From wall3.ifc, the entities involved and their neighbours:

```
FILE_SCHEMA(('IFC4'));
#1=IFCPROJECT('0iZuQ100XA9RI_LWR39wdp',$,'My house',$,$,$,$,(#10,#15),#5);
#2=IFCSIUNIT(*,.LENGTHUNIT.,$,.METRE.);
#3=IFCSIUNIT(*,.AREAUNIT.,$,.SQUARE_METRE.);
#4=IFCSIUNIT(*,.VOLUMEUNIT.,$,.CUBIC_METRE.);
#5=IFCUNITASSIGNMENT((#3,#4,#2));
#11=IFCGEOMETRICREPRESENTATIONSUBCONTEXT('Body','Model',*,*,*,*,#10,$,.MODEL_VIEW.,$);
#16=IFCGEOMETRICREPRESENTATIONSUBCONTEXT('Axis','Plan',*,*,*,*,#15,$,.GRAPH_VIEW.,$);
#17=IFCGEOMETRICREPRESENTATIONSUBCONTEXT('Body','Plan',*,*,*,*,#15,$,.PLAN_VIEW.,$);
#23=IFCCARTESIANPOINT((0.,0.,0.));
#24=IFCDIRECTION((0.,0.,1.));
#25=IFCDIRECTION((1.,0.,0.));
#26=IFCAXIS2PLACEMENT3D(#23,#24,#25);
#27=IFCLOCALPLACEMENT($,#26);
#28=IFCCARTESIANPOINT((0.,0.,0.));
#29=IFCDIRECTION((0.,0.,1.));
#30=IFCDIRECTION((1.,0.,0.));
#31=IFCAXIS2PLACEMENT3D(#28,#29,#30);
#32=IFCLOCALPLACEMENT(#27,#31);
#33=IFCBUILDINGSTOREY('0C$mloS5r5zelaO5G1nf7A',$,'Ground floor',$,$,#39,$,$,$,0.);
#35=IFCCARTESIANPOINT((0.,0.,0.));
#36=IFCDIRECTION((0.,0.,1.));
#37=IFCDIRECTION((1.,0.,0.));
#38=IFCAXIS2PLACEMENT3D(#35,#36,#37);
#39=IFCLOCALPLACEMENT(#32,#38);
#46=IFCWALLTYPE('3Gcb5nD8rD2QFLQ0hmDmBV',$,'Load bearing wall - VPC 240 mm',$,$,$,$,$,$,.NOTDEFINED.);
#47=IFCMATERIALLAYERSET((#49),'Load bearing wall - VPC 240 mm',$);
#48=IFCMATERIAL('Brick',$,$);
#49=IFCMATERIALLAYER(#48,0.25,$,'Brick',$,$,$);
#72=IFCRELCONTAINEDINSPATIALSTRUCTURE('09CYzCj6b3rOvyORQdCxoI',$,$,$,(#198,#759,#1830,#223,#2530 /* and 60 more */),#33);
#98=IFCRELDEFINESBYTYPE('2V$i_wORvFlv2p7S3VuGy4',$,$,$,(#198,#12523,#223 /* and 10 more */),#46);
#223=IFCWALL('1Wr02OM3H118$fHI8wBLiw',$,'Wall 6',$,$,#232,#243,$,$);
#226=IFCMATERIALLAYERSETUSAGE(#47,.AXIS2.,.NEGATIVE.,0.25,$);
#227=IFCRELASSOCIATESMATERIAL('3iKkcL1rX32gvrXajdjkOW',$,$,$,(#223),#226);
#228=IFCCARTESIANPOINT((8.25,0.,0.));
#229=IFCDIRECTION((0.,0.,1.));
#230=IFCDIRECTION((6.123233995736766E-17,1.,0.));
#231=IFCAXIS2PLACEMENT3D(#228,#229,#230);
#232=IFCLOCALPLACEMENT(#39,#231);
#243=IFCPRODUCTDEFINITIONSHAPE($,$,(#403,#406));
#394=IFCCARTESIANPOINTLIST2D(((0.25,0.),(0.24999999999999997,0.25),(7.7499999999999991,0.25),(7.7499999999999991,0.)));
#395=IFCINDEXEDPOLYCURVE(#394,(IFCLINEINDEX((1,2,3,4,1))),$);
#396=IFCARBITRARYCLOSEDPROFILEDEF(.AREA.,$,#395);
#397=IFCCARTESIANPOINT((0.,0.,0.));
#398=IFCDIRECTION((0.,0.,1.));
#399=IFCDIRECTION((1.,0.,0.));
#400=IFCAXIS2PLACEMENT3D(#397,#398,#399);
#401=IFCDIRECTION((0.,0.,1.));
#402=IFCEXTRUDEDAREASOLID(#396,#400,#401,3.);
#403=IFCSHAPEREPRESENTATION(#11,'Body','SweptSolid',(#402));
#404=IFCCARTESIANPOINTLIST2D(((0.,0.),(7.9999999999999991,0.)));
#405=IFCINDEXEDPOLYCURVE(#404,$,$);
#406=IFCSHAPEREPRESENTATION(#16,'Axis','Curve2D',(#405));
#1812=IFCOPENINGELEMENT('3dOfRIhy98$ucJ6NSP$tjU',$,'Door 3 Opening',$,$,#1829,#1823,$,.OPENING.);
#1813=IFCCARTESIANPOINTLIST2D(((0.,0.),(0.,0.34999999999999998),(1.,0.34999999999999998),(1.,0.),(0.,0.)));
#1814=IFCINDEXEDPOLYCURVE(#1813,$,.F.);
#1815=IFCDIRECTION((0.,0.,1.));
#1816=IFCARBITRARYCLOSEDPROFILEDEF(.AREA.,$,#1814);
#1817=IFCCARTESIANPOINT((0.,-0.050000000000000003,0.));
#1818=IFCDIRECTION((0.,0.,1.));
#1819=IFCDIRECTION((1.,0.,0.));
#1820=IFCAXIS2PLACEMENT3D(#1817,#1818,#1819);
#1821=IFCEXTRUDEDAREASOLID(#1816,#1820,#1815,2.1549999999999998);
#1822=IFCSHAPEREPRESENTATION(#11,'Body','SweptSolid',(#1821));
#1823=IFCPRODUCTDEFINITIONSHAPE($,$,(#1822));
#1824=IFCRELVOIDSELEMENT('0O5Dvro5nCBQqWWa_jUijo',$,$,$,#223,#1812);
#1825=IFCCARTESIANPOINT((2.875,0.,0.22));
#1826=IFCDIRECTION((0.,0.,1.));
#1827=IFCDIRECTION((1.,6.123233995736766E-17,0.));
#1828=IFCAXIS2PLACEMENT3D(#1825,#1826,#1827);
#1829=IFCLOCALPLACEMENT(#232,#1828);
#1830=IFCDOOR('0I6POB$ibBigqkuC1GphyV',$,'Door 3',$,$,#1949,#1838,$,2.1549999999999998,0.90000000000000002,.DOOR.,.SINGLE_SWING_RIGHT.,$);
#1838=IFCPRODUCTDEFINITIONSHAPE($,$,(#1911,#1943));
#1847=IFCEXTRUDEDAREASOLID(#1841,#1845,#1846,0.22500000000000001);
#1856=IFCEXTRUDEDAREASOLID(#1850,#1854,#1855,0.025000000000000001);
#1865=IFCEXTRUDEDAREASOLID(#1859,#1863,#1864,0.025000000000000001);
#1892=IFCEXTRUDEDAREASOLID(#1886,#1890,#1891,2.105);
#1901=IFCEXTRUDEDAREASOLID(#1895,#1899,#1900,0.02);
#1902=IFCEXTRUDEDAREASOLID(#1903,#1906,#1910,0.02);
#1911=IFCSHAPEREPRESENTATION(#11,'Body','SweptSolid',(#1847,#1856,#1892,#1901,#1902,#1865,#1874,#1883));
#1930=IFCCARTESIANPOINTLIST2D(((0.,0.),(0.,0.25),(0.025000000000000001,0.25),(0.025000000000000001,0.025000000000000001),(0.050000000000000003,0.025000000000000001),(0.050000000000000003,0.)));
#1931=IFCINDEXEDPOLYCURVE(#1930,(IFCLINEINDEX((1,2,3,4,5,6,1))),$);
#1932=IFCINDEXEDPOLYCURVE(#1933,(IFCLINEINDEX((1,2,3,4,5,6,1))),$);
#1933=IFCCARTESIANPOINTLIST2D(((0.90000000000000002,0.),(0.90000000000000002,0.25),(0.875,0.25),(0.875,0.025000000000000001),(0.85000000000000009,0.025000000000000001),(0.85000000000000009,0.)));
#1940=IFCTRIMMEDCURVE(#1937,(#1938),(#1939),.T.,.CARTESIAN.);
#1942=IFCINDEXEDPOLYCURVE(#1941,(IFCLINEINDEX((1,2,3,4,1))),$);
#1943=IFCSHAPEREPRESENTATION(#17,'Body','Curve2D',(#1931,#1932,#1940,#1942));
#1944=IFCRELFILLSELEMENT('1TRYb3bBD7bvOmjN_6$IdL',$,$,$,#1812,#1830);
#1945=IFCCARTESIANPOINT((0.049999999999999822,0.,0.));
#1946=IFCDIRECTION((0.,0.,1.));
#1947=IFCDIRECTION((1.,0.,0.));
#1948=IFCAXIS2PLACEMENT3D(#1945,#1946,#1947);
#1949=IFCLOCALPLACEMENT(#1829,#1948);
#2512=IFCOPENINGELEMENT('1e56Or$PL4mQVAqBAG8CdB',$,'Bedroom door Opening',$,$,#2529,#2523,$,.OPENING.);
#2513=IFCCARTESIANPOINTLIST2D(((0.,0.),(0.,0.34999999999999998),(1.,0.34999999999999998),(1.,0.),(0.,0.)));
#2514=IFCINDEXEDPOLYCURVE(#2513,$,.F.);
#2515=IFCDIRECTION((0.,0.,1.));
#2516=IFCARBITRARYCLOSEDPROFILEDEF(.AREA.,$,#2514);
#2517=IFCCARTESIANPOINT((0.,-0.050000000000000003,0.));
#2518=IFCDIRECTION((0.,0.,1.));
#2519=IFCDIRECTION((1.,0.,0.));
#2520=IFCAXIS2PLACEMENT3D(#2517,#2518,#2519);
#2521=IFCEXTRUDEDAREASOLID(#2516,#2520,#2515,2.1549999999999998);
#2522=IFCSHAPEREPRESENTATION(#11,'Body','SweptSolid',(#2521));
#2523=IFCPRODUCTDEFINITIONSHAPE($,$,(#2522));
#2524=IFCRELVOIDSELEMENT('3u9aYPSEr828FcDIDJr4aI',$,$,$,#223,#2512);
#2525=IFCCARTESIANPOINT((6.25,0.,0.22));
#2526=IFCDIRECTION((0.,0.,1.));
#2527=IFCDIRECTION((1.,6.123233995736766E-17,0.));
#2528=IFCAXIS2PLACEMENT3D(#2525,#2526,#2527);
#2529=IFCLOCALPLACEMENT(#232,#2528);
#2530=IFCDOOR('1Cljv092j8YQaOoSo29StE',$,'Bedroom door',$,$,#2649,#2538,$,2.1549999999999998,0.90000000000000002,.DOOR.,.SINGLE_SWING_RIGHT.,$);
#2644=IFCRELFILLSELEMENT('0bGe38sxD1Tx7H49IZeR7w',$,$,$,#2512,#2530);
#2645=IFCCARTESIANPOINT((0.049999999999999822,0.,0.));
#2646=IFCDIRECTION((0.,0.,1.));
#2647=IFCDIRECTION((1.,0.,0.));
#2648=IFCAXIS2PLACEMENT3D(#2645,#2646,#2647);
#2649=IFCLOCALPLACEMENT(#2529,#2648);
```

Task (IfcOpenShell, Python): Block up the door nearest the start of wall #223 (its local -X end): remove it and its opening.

```python
import ifcopenshell
import ifcopenshell.api.feature
import ifcopenshell.api.root
import ifcopenshell.geom
import ifcopenshell.util.shape

model = ifcopenshell.open("wall3.ifc")
settings = ifcopenshell.geom.settings()


def volume(element):
    """Net volume in cubic metres, openings subtracted."""
    shape = ifcopenshell.geom.create_shape(settings, element)
    return ifcopenshell.util.shape.get_volume(shape.geometry)


door = model.by_guid("0I6POB$ibBigqkuC1GphyV")
opening = door.FillsVoids[0].RelatingOpeningElement
wall = opening.VoidsElements[0].RelatingBuildingElement
before = volume(wall)

ifcopenshell.api.root.remove_product(model, product=door)
ifcopenshell.api.feature.remove_feature(model, feature=opening)

after = volume(wall)

print(f"wall volume {before:.3f} -> {after:.3f} m3")

model.write("wall3_edited.ifc")
```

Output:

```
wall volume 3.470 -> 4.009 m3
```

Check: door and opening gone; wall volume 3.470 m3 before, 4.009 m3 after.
